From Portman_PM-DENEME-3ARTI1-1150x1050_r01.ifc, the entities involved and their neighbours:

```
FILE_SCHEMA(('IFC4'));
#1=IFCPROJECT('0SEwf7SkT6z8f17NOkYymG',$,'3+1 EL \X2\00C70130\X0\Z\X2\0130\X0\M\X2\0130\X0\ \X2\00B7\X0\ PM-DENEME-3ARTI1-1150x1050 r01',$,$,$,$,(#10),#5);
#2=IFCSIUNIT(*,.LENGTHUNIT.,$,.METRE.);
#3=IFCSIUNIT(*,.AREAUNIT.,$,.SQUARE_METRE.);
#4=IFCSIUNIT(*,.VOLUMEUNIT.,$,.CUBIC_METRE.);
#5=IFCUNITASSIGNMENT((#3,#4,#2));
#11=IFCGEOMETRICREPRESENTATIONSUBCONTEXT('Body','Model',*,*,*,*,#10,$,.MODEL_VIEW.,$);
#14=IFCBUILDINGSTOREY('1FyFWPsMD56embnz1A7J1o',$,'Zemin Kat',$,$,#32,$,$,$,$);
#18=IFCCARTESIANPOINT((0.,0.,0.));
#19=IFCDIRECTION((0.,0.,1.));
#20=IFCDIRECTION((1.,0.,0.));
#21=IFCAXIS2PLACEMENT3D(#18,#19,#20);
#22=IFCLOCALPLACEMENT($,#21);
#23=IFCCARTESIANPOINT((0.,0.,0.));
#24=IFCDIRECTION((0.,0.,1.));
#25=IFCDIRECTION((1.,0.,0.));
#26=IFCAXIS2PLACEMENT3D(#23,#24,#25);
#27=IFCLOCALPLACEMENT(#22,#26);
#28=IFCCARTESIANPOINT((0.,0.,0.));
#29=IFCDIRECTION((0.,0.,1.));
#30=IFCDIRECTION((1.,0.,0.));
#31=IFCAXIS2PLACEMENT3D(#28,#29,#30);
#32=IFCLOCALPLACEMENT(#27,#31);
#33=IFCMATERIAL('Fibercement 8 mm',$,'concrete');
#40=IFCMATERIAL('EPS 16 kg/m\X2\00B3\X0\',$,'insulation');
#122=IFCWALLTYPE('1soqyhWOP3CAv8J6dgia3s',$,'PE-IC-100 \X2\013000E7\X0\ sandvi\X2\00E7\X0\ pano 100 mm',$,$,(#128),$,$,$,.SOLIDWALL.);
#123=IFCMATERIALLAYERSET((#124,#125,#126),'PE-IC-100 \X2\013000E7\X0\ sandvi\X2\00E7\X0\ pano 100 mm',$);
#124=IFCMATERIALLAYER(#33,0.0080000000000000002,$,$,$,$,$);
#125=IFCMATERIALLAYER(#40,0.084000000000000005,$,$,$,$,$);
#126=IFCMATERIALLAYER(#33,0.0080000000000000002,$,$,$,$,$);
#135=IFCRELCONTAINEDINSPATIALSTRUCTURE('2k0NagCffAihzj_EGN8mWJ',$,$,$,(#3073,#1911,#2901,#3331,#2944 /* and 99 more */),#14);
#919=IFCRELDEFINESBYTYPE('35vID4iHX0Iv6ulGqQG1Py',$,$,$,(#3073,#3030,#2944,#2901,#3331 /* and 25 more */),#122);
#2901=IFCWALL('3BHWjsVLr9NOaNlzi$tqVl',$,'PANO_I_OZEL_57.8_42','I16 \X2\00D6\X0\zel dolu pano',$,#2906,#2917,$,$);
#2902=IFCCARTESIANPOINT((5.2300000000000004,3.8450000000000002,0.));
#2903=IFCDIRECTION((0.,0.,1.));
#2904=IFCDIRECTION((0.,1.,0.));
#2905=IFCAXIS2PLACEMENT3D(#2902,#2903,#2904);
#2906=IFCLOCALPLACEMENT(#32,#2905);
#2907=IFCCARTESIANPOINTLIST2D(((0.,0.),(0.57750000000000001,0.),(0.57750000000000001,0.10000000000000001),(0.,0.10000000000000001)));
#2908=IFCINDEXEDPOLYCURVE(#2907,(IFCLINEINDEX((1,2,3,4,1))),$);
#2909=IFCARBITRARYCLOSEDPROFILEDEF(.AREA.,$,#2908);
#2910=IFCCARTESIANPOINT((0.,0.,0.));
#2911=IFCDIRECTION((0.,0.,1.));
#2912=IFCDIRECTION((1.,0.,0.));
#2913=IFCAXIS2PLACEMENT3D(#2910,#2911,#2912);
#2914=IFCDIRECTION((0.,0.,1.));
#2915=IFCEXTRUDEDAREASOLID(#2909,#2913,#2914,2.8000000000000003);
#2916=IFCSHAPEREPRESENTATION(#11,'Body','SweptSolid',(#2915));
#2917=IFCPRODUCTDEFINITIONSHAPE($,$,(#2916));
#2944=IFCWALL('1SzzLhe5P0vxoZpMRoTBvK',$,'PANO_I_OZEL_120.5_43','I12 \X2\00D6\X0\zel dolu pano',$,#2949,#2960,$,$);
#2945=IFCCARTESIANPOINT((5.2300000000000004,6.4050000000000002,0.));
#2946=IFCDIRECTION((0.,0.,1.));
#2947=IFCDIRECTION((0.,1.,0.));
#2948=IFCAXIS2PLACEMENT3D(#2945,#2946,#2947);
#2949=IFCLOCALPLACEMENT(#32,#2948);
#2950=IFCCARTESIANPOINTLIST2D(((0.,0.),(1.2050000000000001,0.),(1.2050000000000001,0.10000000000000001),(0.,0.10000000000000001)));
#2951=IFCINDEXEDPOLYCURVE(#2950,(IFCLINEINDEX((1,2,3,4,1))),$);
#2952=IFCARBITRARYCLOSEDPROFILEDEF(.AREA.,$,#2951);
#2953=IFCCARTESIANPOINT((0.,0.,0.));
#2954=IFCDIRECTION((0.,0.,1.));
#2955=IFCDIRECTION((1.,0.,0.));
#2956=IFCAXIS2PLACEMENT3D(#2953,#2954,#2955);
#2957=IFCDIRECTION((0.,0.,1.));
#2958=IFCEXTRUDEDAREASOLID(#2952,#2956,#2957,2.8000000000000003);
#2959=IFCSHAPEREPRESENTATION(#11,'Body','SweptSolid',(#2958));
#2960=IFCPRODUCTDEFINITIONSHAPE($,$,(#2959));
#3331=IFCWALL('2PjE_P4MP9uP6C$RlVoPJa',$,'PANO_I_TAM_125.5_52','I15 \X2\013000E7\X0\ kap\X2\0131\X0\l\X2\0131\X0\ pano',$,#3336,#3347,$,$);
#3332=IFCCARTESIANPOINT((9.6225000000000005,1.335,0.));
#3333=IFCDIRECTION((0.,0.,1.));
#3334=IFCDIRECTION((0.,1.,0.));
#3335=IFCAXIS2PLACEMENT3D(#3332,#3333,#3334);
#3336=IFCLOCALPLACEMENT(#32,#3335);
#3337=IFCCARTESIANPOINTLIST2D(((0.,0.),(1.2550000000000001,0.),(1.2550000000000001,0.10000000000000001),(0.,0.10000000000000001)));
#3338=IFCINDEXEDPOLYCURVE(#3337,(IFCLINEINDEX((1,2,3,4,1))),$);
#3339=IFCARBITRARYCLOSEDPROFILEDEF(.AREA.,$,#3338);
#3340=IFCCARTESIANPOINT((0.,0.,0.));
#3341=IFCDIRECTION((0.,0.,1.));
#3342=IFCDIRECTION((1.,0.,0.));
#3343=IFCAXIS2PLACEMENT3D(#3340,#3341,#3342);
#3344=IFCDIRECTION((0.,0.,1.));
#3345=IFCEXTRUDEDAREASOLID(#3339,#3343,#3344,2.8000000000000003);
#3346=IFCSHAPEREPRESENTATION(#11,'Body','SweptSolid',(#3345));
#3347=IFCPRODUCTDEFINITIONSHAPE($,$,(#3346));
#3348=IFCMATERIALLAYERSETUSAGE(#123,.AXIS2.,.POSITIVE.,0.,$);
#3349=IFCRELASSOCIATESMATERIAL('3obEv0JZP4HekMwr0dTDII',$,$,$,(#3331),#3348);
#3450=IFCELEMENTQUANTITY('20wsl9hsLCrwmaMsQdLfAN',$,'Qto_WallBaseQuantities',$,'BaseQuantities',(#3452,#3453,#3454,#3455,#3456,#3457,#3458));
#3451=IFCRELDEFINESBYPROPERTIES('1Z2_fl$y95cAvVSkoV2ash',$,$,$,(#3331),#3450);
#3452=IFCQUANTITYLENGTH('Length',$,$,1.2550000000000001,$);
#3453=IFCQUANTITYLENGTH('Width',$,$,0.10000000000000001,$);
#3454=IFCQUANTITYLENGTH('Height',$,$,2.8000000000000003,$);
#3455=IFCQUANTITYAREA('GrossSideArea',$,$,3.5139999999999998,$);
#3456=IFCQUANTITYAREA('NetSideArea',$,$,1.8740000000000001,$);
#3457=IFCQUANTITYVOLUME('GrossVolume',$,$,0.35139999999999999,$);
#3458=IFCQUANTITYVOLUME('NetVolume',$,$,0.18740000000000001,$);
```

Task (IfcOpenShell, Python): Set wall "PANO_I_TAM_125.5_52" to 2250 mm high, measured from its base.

```python
import ifcopenshell
import ifcopenshell.api.pset
import ifcopenshell.geom
import ifcopenshell.util.element
import ifcopenshell.util.representation
import ifcopenshell.util.shape
import ifcopenshell.util.unit

model = ifcopenshell.open("Portman_PM-DENEME-3ARTI1-1150x1050_r01.ifc")
unit_scale = ifcopenshell.util.unit.calculate_unit_scale(model)
area_scale = ifcopenshell.util.unit.calculate_unit_scale(model, "AREAUNIT")
volume_scale = ifcopenshell.util.unit.calculate_unit_scale(model, "VOLUMEUNIT")
settings = ifcopenshell.geom.settings()


def volume(element):
    """Net volume in cubic metres, openings subtracted."""
    shape = ifcopenshell.geom.create_shape(settings, element)
    return ifcopenshell.util.shape.get_volume(shape.geometry)


wall = model.by_guid("2PjE_P4MP9uP6C$RlVoPJa")
before = volume(wall)

body = ifcopenshell.util.representation.get_representation(wall, "Model", "Body")
solid = body.Items[0]
old_height = solid.Depth
solid.Depth = 2.25 / unit_scale
after = volume(wall)
thickness = 0.1  # wall thickness in metres

# Update the stored height, areas and volumes.
qto = model.by_id(ifcopenshell.util.element.get_pset(wall, "Qto_WallBaseQuantities", should_inherit=False)["id"])
ifcopenshell.api.pset.edit_qto(model, qto=qto, properties={
    "Height": solid.Depth,
    "GrossSideArea": ifcopenshell.util.element.get_pset(wall, "Qto_WallBaseQuantities", "GrossSideArea") * solid.Depth / old_height,
    "NetSideArea": after / thickness / area_scale,
    "GrossVolume": ifcopenshell.util.element.get_pset(wall, "Qto_WallBaseQuantities", "GrossVolume") * solid.Depth / old_height,
    "NetVolume": after / volume_scale,
})

print(f"height {old_height:g} -> {solid.Depth:g}, volume {before:.3f} -> {after:.3f} m3")

model.write("Portman_PM-DENEME-3ARTI1-1150x1050_r01_edited.ifc")
```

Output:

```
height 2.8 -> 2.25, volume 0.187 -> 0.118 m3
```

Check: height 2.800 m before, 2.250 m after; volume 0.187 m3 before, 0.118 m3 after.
